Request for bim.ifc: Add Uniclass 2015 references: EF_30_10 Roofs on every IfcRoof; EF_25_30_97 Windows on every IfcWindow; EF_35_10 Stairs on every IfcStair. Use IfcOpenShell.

First a look at what the model holds.

```python
import ifcopenshell

model = ifcopenshell.open("bim.ifc")
print(model.schema)
print("classifications:", [c.Name for c in model.by_type("IfcClassification")])
for ifc_class in ("IfcDoor", "IfcRoof", "IfcStair", "IfcWall", "IfcWindow"):
    print(ifc_class, len(model.by_type(ifc_class)))
```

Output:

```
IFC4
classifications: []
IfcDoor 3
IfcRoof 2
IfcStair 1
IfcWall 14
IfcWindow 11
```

```python
import ifcopenshell
import ifcopenshell.api.classification

model = ifcopenshell.open("bim.ifc")

system = ifcopenshell.api.classification.add_classification(model, classification="Uniclass 2015")

codes = {
    "IfcRoof": ("EF_30_10", "Roofs"),
    "IfcWindow": ("EF_25_30_97", "Windows"),
    "IfcStair": ("EF_35_10", "Stairs"),
}
for ifc_class, (code, name) in codes.items():
    products = model.by_type(ifc_class)
    ifcopenshell.api.classification.add_reference(
        model, products=products, classification=system, identification=code, name=name
    )
    print(code, len(products))

model.write("bim_rev.ifc")
```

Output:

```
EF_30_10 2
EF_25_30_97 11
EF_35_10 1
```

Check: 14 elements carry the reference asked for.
